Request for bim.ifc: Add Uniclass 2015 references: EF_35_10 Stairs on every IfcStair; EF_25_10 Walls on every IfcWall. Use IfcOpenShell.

First a look at what the model holds.

```python
import ifcopenshell

model = ifcopenshell.open("bim.ifc")
print(model.schema)
print("classifications:", [c.Name for c in model.by_type("IfcClassification")])
for ifc_class in ("IfcDoor", "IfcRoof", "IfcStair", "IfcWall", "IfcWindow"):
    print(ifc_class, len(model.by_type(ifc_class)))
```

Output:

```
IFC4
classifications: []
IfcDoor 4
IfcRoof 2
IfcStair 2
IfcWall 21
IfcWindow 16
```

```python
import ifcopenshell
import ifcopenshell.api.classification

model = ifcopenshell.open("bim.ifc")

system = ifcopenshell.api.classification.add_classification(model, classification="Uniclass 2015")

codes = {
    "IfcStair": ("EF_35_10", "Stairs"),
    "IfcWall": ("EF_25_10", "Walls"),
}
for ifc_class, (code, name) in codes.items():
    products = model.by_type(ifc_class)
    ifcopenshell.api.classification.add_reference(
        model, products=products, classification=system, identification=code, name=name
    )
    print(code, len(products))

model.write("bim-out.ifc")
```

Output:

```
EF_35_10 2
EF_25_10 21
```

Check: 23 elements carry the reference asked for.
